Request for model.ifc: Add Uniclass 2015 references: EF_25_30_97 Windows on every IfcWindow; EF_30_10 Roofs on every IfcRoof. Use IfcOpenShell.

First a look at what the model holds.

```python
import ifcopenshell

model = ifcopenshell.open("model.ifc")
print(model.schema)
print("classifications:", [c.Name for c in model.by_type("IfcClassification")])
for ifc_class in ("IfcDoor", "IfcRoof", "IfcStair", "IfcWall", "IfcWindow"):
    print(ifc_class, len(model.by_type(ifc_class)))
```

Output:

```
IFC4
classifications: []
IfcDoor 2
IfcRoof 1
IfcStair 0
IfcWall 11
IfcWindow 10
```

```python
import ifcopenshell
import ifcopenshell.api.classification

model = ifcopenshell.open("model.ifc")

system = ifcopenshell.api.classification.add_classification(model, classification="Uniclass 2015")

codes = {
    "IfcWindow": ("EF_25_30_97", "Windows"),
    "IfcRoof": ("EF_30_10", "Roofs"),
}
for ifc_class, (code, name) in codes.items():
    products = model.by_type(ifc_class)
    ifcopenshell.api.classification.add_reference(
        model, products=products, classification=system, identification=code, name=name
    )
    print(code, len(products))

model.write("model_edited.ifc")
```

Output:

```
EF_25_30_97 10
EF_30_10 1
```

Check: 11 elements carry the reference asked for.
